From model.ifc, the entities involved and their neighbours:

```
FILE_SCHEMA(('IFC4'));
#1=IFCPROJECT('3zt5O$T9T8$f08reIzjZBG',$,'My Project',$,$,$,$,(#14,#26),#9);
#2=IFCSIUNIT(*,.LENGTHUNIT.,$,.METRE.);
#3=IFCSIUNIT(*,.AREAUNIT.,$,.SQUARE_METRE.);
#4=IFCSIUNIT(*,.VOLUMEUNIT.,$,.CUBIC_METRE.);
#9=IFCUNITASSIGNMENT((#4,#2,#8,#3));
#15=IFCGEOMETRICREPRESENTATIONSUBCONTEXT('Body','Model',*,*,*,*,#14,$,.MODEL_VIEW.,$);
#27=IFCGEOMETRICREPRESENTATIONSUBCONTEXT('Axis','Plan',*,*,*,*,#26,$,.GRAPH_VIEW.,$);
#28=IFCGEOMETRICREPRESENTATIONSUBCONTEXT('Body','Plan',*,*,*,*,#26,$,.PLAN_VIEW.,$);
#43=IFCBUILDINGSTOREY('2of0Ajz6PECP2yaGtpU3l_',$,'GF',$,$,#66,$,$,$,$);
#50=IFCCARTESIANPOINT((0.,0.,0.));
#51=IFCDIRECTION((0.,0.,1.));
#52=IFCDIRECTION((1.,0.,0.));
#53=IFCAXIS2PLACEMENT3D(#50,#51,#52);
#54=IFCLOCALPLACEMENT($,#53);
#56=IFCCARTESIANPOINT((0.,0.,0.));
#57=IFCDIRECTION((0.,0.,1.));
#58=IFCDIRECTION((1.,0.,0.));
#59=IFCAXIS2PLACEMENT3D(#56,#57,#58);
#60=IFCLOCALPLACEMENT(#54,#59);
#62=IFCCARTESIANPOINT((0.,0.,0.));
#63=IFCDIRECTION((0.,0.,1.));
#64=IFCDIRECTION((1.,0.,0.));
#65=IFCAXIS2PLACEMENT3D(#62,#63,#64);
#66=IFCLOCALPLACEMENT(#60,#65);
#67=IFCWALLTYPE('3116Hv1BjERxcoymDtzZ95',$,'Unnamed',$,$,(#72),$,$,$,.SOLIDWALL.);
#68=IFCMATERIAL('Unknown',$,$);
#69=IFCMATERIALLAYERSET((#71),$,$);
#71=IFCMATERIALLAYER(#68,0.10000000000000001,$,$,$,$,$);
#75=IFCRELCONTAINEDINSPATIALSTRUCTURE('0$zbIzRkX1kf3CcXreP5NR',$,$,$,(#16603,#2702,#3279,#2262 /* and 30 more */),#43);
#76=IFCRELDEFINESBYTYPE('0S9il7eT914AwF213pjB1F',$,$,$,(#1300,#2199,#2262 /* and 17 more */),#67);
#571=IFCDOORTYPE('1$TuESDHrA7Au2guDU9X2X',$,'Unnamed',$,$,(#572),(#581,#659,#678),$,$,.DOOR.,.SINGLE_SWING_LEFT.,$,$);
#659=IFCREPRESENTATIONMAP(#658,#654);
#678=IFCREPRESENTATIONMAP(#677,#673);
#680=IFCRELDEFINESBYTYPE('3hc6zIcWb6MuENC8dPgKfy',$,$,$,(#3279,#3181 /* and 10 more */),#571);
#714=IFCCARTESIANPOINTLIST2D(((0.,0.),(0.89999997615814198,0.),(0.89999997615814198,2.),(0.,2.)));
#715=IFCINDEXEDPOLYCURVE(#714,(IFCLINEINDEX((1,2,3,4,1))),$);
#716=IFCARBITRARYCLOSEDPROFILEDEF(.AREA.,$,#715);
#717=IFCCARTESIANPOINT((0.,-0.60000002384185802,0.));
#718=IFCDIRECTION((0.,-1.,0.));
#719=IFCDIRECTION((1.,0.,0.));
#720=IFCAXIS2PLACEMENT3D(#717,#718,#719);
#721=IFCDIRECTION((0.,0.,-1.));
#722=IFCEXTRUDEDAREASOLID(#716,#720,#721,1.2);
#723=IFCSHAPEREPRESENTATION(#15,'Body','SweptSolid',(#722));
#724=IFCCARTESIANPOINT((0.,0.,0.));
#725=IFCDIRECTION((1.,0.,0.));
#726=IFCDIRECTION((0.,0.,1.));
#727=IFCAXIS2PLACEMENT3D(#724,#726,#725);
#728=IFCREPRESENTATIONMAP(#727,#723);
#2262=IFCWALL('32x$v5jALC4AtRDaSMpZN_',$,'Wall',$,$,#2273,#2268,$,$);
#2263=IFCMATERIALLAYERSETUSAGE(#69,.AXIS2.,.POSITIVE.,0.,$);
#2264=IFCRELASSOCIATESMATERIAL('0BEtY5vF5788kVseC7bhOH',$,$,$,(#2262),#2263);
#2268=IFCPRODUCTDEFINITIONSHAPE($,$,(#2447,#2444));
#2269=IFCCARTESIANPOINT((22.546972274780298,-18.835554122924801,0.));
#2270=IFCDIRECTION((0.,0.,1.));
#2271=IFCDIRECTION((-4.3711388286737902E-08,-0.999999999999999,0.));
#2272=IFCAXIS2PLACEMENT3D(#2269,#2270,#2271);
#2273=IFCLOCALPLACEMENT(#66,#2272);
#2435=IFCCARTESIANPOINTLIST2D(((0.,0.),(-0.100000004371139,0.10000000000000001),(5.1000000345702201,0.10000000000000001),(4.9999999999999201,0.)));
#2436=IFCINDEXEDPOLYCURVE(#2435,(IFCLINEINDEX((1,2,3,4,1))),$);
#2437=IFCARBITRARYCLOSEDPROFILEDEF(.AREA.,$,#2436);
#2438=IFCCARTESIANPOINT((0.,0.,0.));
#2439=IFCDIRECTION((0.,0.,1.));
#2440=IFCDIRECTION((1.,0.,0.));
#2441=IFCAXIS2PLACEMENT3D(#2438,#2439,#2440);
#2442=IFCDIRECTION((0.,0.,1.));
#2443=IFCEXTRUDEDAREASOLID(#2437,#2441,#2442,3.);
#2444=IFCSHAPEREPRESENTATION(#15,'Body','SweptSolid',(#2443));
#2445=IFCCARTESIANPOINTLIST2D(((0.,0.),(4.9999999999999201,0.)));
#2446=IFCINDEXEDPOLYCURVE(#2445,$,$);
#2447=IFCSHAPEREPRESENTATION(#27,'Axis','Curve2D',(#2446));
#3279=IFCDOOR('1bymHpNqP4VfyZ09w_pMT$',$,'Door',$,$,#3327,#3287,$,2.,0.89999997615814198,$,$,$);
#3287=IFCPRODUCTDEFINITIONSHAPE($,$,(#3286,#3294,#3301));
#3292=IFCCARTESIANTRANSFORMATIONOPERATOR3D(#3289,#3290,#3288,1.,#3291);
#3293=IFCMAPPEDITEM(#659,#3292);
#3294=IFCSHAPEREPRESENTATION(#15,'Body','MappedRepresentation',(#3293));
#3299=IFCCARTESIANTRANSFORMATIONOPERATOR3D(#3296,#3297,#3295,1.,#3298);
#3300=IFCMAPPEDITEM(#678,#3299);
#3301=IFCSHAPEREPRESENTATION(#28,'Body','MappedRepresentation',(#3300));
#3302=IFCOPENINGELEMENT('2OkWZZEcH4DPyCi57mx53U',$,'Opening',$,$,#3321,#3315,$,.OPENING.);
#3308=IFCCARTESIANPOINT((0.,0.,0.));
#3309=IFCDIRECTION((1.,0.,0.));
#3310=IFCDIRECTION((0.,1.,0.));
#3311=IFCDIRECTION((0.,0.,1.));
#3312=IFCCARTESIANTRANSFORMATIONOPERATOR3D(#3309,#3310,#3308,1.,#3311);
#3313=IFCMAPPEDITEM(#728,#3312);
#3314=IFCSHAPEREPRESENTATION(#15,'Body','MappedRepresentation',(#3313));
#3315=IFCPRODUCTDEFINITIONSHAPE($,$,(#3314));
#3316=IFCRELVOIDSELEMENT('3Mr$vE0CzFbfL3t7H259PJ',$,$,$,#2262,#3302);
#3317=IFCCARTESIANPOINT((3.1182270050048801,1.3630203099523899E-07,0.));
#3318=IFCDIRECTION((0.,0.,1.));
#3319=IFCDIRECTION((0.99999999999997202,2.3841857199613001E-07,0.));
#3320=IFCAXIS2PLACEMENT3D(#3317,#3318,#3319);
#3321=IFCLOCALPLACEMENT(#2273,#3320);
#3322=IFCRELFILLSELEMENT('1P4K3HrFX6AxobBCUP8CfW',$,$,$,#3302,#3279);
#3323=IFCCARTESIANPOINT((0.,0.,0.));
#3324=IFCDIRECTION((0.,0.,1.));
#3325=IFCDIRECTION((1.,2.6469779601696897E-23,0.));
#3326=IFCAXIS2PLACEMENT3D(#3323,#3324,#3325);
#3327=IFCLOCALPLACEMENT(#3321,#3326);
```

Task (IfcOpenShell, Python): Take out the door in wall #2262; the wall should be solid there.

```python
import ifcopenshell
import ifcopenshell.api.feature
import ifcopenshell.api.root
import ifcopenshell.geom
import ifcopenshell.util.shape

model = ifcopenshell.open("model.ifc")
settings = ifcopenshell.geom.settings()


def volume(element):
    """Net volume in cubic metres, openings subtracted."""
    shape = ifcopenshell.geom.create_shape(settings, element)
    return ifcopenshell.util.shape.get_volume(shape.geometry)


door = model.by_guid("1bymHpNqP4VfyZ09w_pMT$")
opening = door.FillsVoids[0].RelatingOpeningElement
wall = opening.VoidsElements[0].RelatingBuildingElement
before = volume(wall)

ifcopenshell.api.root.remove_product(model, product=door)
ifcopenshell.api.feature.remove_feature(model, feature=opening)

after = volume(wall)

print(f"wall volume {before:.3f} -> {after:.3f} m3")

model.write("model_v2.ifc")
```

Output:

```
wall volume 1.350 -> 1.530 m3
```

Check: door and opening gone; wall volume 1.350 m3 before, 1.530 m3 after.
